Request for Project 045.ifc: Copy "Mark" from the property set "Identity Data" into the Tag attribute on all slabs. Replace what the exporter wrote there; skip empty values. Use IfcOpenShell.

First a look at what the model holds.

```python
import ifcopenshell
import ifcopenshell.util.element

model = ifcopenshell.open("Project 045.ifc")
print(model.schema)
slabs = model.by_type("IfcSlab")
print(len(slabs), "slabs")
for e in slabs[:8]:
    source = ifcopenshell.util.element.get_pset(e, "Identity Data", "Mark")
    target = e.Tag
    print(e.id(), repr(source), repr(target), sep=" | ")
```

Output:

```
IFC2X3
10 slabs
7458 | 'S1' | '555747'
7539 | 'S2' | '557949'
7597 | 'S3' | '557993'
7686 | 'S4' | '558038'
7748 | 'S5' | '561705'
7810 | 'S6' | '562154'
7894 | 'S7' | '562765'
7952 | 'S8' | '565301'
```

```python
import ifcopenshell
import ifcopenshell.util.element

model = ifcopenshell.open("Project 045.ifc")

count = 0
for e in model.by_type("IfcSlab"):
    value = ifcopenshell.util.element.get_pset(e, "Identity Data", "Mark")
    current = e.Tag
    if not value or not value.strip() or current == value:
        continue
    e.Tag = value
    count += 1

print(count, "slabs updated")

model.write("Project 045_edited.ifc")
```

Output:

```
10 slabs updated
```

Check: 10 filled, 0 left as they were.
